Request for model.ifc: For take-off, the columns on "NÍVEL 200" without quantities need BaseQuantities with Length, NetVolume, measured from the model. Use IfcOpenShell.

First a look at what the model holds.

```python
import ifcopenshell
import ifcopenshell.util.element
import ifcopenshell.util.unit

model = ifcopenshell.open("model.ifc")
print(model.schema)
for unit_type in ("LENGTHUNIT", "AREAUNIT", "VOLUMEUNIT"):
    print(unit_type, ifcopenshell.util.unit.calculate_unit_scale(model, unit_type))
storey = next(s for s in model.by_type("IfcBuildingStorey") if s.Name == "NÍVEL 200")
columns = [e for e in ifcopenshell.util.element.get_decomposition(storey) if e.is_a("IfcColumn")]
for e in sorted(columns, key=lambda e: e.id()):
    print(e.id(), e.is_a(), e.Name, list(ifcopenshell.util.element.get_psets(e, qtos_only=True)), sep=" | ")
```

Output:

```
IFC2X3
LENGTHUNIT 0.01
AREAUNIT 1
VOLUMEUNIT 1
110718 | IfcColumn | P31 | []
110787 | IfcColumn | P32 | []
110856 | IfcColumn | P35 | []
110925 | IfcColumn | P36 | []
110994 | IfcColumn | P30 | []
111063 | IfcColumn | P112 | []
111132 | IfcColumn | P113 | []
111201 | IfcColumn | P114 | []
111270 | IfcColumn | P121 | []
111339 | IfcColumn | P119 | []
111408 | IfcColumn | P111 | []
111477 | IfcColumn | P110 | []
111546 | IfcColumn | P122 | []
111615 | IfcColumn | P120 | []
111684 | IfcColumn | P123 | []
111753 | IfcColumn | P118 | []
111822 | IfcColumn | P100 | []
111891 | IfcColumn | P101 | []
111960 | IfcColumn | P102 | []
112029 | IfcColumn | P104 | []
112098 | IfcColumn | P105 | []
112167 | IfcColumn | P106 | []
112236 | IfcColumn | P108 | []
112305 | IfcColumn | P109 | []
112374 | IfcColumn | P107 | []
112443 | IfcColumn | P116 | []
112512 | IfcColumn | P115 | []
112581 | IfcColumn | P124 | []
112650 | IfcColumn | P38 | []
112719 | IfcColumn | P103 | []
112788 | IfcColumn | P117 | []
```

```python
import ifcopenshell
import ifcopenshell.api.pset
import ifcopenshell.geom
import ifcopenshell.util.element
import ifcopenshell.util.shape
import ifcopenshell.util.unit

model = ifcopenshell.open("model.ifc")
unit_scale = ifcopenshell.util.unit.calculate_unit_scale(model)
volume_scale = ifcopenshell.util.unit.calculate_unit_scale(model, "VOLUMEUNIT")
settings = ifcopenshell.geom.settings()

storey = next(s for s in model.by_type("IfcBuildingStorey") if s.Name == "NÍVEL 200")
columns = [e for e in ifcopenshell.util.element.get_decomposition(storey) if e.is_a("IfcColumn")]

for e in sorted(columns, key=lambda e: e.id()):
    if ifcopenshell.util.element.get_psets(e, qtos_only=True, should_inherit=False):
        continue
    # Geometry comes back in metres, in the element's own axes.
    shape = ifcopenshell.geom.create_shape(settings, e)
    values = {
        "Length": ifcopenshell.util.shape.get_z(shape.geometry) / unit_scale,
        "NetVolume": ifcopenshell.util.shape.get_volume(shape.geometry) / volume_scale,
    }
    qto = ifcopenshell.api.pset.add_qto(model, product=e, name="BaseQuantities")
    ifcopenshell.api.pset.edit_qto(model, qto=qto, properties=values)
    print(e.id(), {k: round(v, 3) for k, v in values.items()})

model.write("model_updated.ifc")
```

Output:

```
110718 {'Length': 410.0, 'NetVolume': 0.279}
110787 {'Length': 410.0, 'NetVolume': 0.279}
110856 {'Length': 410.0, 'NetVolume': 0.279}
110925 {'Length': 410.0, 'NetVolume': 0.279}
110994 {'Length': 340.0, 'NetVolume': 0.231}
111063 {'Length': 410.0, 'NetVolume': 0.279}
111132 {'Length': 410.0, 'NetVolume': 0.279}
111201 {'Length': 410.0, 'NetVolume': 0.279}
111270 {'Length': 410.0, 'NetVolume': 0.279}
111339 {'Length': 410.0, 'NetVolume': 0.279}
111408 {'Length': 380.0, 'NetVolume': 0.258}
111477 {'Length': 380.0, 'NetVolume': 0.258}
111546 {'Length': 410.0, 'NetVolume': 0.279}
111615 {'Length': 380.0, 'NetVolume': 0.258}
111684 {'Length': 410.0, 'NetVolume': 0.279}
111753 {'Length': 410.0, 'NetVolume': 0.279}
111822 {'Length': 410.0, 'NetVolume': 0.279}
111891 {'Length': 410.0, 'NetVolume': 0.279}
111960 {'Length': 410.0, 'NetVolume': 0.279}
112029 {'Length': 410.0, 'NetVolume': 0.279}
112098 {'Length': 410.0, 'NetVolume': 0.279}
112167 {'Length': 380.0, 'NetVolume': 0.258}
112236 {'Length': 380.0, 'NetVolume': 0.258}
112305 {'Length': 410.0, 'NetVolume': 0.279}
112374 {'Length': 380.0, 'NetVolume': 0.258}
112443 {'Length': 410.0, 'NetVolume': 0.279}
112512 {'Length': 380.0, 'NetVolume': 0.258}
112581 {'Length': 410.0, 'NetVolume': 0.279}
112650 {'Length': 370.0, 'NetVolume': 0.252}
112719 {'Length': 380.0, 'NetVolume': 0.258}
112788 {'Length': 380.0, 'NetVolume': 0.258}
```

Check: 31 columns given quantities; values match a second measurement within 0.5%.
